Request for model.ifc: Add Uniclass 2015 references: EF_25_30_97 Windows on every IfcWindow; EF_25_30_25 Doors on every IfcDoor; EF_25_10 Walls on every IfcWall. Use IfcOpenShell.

First a look at what the model holds.

```python
import ifcopenshell

model = ifcopenshell.open("model.ifc")
print(model.schema)
print("classifications:", [c.Name for c in model.by_type("IfcClassification")])
for ifc_class in ("IfcDoor", "IfcRoof", "IfcStair", "IfcWall", "IfcWindow"):
    print(ifc_class, len(model.by_type(ifc_class)))
```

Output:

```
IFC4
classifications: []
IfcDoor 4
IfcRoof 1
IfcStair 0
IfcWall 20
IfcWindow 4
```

```python
import ifcopenshell
import ifcopenshell.api.classification

model = ifcopenshell.open("model.ifc")

system = ifcopenshell.api.classification.add_classification(model, classification="Uniclass 2015")

codes = {
    "IfcWindow": ("EF_25_30_97", "Windows"),
    "IfcDoor": ("EF_25_30_25", "Doors"),
    "IfcWall": ("EF_25_10", "Walls"),
}
for ifc_class, (code, name) in codes.items():
    products = model.by_type(ifc_class)
    ifcopenshell.api.classification.add_reference(
        model, products=products, classification=system, identification=code, name=name
    )
    print(code, len(products))

model.write("model_updated.ifc")
```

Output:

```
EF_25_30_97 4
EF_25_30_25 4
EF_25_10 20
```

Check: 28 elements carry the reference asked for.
